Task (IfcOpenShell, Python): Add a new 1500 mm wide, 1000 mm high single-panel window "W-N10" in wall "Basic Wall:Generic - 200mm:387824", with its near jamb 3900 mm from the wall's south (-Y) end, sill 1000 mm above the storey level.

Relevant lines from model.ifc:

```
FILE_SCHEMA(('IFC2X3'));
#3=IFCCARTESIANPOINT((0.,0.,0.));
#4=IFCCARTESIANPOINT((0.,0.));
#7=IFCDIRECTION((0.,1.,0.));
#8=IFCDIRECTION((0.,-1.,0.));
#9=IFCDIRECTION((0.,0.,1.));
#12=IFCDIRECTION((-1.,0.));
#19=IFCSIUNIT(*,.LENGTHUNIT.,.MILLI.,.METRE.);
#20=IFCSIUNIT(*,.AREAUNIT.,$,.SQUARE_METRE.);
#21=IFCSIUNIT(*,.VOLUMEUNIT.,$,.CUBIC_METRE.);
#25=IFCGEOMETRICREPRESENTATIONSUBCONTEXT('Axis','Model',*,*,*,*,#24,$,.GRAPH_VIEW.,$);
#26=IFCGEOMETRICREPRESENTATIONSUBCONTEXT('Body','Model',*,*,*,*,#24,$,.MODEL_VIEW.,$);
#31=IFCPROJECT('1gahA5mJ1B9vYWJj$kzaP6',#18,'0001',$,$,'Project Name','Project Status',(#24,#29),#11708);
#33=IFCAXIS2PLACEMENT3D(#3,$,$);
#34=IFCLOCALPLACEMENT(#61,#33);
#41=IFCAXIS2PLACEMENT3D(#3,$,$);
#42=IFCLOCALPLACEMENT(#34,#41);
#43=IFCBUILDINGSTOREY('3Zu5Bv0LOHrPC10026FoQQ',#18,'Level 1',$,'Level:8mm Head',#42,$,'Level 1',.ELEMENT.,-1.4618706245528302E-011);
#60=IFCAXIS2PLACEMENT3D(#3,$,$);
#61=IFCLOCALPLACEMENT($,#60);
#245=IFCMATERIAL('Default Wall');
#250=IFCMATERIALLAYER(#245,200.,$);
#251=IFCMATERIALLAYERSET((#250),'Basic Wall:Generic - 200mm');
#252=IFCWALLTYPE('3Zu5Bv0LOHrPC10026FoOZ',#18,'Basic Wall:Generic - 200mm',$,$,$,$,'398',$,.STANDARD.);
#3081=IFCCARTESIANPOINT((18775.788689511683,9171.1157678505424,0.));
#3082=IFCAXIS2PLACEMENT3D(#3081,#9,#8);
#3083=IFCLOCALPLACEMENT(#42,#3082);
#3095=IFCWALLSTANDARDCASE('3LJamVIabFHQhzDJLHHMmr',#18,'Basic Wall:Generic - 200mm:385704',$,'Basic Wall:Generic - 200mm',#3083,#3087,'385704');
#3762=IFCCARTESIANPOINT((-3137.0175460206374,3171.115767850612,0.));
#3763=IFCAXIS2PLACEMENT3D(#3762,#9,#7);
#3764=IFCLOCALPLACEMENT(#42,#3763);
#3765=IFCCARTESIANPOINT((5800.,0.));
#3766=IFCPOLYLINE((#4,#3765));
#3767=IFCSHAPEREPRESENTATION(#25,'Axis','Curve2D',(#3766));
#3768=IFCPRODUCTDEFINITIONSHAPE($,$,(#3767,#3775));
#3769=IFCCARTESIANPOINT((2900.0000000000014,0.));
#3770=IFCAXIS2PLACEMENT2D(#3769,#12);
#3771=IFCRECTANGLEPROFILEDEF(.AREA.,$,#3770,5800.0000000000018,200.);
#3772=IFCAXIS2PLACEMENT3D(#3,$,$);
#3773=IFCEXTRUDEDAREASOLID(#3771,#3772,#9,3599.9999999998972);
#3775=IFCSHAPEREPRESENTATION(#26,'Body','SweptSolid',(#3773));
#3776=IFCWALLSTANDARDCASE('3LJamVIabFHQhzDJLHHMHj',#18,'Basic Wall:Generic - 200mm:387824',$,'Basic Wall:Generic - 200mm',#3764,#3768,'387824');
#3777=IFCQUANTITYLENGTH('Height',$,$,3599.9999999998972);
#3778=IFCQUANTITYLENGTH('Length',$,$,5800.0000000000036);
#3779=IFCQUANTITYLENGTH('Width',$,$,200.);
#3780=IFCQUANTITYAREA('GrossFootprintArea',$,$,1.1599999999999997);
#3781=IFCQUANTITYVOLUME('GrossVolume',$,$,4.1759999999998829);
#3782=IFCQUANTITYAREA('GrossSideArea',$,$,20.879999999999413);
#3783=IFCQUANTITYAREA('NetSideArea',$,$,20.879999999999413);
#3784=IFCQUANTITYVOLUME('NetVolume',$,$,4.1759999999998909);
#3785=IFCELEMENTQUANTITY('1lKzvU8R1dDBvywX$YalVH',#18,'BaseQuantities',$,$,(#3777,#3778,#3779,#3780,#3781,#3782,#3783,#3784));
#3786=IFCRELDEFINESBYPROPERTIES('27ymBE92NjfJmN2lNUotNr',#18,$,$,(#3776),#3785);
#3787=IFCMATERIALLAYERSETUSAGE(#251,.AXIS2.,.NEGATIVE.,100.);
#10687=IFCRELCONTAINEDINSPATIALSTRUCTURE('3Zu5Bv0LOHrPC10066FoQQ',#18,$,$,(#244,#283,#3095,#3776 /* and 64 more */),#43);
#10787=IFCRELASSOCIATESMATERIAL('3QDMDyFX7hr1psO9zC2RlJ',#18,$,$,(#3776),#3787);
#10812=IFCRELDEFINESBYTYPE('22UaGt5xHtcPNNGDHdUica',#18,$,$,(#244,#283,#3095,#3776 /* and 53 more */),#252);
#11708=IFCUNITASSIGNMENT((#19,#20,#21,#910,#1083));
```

```python
import numpy as np
import ifcopenshell
import ifcopenshell.api.feature
import ifcopenshell.api.geometry
import ifcopenshell.api.pset
import ifcopenshell.api.root
import ifcopenshell.api.spatial
import ifcopenshell.api.type
import ifcopenshell.geom
import ifcopenshell.util.element
import ifcopenshell.util.placement
import ifcopenshell.util.representation
import ifcopenshell.util.shape
import ifcopenshell.util.unit

model = ifcopenshell.open("model.ifc")
unit_scale = ifcopenshell.util.unit.calculate_unit_scale(model)
area_scale = ifcopenshell.util.unit.calculate_unit_scale(model, "AREAUNIT")
volume_scale = ifcopenshell.util.unit.calculate_unit_scale(model, "VOLUMEUNIT")
settings = ifcopenshell.geom.settings()


def volume(element):
    """Net volume in cubic metres, openings subtracted."""
    shape = ifcopenshell.geom.create_shape(settings, element)
    return ifcopenshell.util.shape.get_volume(shape.geometry)


wall = model.by_id(3776)
storey = ifcopenshell.util.element.get_container(wall, ifc_class="IfcBuildingStorey")
context = ifcopenshell.util.representation.get_context(model, "Model", "Body", "MODEL_VIEW")
before = volume(wall)

width, height, from_end, sill = 1.5, 1, 3.9, 1  # metres

# The wall runs along its own X axis, and the end named is its -X end.
wall_shape = ifcopenshell.geom.create_shape(settings, wall)
x, y, z = ifcopenshell.util.shape.get_vertices(wall_shape.geometry).T
start = x.min() + from_end
face, thickness = float(y.min()), float(y.max() - y.min())
wall_matrix = ifcopenshell.util.placement.get_local_placement(wall.ObjectPlacement)
level = ifcopenshell.util.placement.get_local_placement(storey.ObjectPlacement)[2, 3]


def in_wall(x, y):
    """Placement at x, y metres in the wall's axes, at sill height."""
    matrix = wall_matrix.copy()
    matrix[:, 3] = wall_matrix @ np.array([x / unit_scale, y / unit_scale, 0.0, 1.0])
    matrix[2, 3] = level + sill / unit_scale
    return matrix


# Opening: a box that overshoots both wall faces by 50 mm.
opening = ifcopenshell.api.root.create_entity(model, ifc_class="IfcOpeningElement")
box = ifcopenshell.api.geometry.add_wall_representation(
    model, context=context, length=width, height=height, thickness=thickness + 0.1
)
ifcopenshell.api.geometry.assign_representation(model, product=opening, representation=box)
ifcopenshell.api.geometry.edit_object_placement(model, product=opening, matrix=in_wall(start, face - 0.05), is_si=False)
ifcopenshell.api.feature.add_feature(model, feature=opening, element=wall)

window = ifcopenshell.api.root.create_entity(model, ifc_class="IfcWindow", name="W-N10")
window.OverallWidth, window.OverallHeight = width / unit_scale, height / unit_scale
body = ifcopenshell.api.geometry.add_window_representation(
    model,
    context=context,
    overall_width=window.OverallWidth,
    overall_height=window.OverallHeight,
    partition_type="SINGLE_PANEL",
)
ifcopenshell.api.geometry.assign_representation(model, product=window, representation=body)
ifcopenshell.api.spatial.assign_container(model, products=[window], relating_structure=storey)
fills = ifcopenshell.api.feature.add_filling(model, opening=opening, element=window)
fills.OwnerHistory = window.OwnerHistory  # required in IFC2X3

# IFC2X3 keeps the operation on the window style.
style = ifcopenshell.api.root.create_entity(model, ifc_class="IfcWindowStyle", name="W-N10")
style.OperationType, style.ConstructionType = "SINGLE_PANEL", "NOTDEFINED"
style.ParameterTakesPrecedence = style.Sizeable = False
ifcopenshell.api.type.assign_type(model, related_objects=[window], relating_type=style)

# Centre the window in the wall's thickness.
ifcopenshell.api.geometry.edit_object_placement(model, product=window, matrix=in_wall(start, face), is_si=False)
window_shape = ifcopenshell.geom.create_shape(settings, window)
depth = ifcopenshell.util.shape.get_vertices(window_shape.geometry)[:, 1]
offset = face + thickness / 2 - (depth.min() + depth.max()) / 2
ifcopenshell.api.geometry.edit_object_placement(model, product=window, matrix=in_wall(start, offset), is_si=False)

after = volume(wall)

# Update the wall's stored quantities.
qto = model.by_id(ifcopenshell.util.element.get_pset(wall, "BaseQuantities", should_inherit=False)["id"])
ifcopenshell.api.pset.edit_qto(model, qto=qto, properties={
    "NetSideArea": after / thickness / area_scale,
    "NetVolume": after / volume_scale,
})

print(f"wall volume {before:.3f} -> {after:.3f} m3")

model.write("model-out.ifc")
```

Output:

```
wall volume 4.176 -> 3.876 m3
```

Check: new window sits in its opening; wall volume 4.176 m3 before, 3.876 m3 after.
